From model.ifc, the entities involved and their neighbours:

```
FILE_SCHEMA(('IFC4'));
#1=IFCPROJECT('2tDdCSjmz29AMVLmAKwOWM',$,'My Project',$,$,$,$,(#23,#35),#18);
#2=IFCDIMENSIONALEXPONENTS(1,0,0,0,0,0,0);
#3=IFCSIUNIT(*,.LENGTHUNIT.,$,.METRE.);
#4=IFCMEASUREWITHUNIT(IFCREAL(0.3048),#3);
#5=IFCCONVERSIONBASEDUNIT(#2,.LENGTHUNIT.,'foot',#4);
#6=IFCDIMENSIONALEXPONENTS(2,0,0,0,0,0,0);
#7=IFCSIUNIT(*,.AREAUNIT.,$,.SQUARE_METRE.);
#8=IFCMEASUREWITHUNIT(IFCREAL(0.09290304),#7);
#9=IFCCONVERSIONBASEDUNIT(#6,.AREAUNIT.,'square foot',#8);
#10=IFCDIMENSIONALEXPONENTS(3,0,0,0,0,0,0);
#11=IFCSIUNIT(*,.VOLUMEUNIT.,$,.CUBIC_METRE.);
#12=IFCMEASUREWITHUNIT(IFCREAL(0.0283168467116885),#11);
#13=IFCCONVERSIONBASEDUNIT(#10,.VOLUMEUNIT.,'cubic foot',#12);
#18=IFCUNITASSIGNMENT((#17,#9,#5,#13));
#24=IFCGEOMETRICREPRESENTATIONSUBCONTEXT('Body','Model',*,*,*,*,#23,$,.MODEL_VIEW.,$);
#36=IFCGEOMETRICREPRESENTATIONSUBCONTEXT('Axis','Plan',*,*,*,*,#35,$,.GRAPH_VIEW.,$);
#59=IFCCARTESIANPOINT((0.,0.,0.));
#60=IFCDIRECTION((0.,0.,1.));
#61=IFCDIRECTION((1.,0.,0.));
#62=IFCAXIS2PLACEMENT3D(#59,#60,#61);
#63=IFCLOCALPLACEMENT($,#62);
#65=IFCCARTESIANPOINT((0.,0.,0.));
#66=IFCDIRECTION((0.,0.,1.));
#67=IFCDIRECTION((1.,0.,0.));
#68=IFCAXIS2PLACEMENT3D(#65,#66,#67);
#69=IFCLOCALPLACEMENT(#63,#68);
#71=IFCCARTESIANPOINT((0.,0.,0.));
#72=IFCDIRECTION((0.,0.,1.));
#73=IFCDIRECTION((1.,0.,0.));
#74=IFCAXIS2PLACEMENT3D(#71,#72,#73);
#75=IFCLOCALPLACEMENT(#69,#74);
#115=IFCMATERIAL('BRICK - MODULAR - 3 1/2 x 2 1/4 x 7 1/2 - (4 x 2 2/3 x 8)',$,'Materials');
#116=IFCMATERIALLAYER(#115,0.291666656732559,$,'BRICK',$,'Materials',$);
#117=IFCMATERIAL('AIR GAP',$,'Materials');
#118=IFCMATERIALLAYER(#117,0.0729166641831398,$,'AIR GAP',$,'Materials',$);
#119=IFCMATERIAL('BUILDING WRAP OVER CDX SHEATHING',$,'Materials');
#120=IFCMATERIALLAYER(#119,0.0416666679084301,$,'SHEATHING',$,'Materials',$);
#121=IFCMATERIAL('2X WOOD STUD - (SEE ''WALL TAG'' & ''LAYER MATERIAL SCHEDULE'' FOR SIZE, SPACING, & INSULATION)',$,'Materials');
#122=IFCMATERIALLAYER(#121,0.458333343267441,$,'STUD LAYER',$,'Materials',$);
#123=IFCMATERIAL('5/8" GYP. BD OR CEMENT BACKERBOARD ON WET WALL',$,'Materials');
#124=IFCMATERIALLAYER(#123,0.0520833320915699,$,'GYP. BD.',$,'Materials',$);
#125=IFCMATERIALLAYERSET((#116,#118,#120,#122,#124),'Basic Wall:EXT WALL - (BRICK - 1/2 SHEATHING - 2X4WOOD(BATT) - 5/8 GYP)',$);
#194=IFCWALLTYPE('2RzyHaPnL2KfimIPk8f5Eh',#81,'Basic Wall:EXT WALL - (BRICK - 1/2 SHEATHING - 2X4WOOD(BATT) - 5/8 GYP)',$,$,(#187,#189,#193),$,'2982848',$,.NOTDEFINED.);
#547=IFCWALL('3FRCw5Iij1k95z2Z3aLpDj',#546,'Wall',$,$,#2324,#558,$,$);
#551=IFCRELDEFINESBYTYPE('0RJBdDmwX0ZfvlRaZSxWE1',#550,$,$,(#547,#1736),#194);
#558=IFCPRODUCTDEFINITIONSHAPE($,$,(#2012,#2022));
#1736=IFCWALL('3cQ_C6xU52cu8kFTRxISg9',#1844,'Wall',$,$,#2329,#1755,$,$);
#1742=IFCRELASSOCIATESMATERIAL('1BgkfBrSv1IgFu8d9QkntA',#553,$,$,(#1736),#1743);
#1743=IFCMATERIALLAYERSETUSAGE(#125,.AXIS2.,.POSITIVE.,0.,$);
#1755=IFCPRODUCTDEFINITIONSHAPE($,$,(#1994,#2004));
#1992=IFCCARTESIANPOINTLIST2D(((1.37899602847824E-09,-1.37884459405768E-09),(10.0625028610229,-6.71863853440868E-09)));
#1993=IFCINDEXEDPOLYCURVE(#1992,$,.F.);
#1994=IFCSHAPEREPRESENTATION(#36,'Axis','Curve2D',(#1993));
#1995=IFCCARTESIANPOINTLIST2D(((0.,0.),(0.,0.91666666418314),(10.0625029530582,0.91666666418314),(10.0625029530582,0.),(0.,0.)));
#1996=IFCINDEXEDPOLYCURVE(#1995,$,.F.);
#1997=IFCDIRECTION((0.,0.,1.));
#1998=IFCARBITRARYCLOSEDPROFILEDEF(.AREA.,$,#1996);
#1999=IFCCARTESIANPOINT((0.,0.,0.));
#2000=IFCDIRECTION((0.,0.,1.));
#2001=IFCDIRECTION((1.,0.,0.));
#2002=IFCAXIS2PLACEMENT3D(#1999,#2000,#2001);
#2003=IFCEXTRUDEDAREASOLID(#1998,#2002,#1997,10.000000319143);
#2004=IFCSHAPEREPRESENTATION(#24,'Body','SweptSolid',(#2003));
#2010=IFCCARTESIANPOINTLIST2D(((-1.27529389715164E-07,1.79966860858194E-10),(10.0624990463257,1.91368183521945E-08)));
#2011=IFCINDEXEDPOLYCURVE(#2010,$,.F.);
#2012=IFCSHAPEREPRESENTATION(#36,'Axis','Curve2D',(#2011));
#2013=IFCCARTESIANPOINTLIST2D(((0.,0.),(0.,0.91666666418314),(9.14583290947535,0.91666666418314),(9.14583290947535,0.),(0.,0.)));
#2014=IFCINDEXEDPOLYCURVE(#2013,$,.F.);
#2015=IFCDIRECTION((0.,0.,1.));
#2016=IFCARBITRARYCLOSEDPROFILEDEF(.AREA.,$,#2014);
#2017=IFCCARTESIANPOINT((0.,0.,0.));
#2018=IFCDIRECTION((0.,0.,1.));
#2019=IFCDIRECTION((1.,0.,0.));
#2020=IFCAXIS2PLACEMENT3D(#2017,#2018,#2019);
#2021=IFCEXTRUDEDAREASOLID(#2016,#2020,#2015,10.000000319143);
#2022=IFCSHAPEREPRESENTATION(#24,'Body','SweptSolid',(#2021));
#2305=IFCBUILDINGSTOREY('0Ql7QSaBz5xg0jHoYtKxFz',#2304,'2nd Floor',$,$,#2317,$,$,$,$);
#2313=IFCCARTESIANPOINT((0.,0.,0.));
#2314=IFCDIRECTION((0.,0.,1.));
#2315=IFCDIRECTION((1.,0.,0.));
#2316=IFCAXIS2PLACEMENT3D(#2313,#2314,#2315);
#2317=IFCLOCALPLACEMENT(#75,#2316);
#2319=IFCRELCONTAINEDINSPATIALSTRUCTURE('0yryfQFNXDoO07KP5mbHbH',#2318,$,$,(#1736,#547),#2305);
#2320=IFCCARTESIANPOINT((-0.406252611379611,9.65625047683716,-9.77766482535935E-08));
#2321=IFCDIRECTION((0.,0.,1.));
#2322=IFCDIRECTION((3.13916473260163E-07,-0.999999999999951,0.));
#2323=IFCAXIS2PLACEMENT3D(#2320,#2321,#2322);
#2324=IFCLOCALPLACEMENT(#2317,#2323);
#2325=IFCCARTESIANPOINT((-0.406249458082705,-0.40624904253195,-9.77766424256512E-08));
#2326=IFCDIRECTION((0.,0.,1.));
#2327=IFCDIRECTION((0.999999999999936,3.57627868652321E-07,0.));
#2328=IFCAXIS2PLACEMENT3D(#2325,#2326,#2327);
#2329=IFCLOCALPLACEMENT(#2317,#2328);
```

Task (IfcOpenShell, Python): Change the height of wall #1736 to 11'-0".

```python
import ifcopenshell
import ifcopenshell.geom
import ifcopenshell.util.representation
import ifcopenshell.util.shape
import ifcopenshell.util.unit

model = ifcopenshell.open("model.ifc")
unit_scale = ifcopenshell.util.unit.calculate_unit_scale(model)
settings = ifcopenshell.geom.settings()


def volume(element):
    """Net volume in cubic metres, openings subtracted."""
    shape = ifcopenshell.geom.create_shape(settings, element)
    return ifcopenshell.util.shape.get_volume(shape.geometry)


wall = model.by_id(1736)
before = volume(wall)

body = ifcopenshell.util.representation.get_representation(wall, "Model", "Body")
solid = body.Items[0]
old_height = solid.Depth
solid.Depth = 132 * 0.0254 / unit_scale
after = volume(wall)

print(f"height {old_height:g} -> {solid.Depth:g}, volume {before:.3f} -> {after:.3f} m3")

model.write("model_rev.ifc")
```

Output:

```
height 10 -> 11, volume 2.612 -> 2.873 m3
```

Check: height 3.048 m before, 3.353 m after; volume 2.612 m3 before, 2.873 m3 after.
